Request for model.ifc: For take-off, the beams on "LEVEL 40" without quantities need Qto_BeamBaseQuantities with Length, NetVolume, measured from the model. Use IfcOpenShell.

First a look at what the model holds.

```python
import ifcopenshell
import ifcopenshell.util.element
import ifcopenshell.util.unit

model = ifcopenshell.open("model.ifc")
print(model.schema)
for unit_type in ("LENGTHUNIT", "AREAUNIT", "VOLUMEUNIT"):
    print(unit_type, ifcopenshell.util.unit.calculate_unit_scale(model, unit_type))
storey = next(s for s in model.by_type("IfcBuildingStorey") if s.Name == "LEVEL 40")
beams = [e for e in ifcopenshell.util.element.get_decomposition(storey) if e.is_a("IfcBeam")]
for e in sorted(beams, key=lambda e: e.id()):
    print(e.id(), e.is_a(), e.Name, list(ifcopenshell.util.element.get_psets(e, qtos_only=True)), sep=" | ")
```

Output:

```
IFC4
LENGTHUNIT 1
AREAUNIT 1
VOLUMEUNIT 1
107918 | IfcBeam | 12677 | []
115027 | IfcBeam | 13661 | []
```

```python
import ifcopenshell
import ifcopenshell.api.pset
import ifcopenshell.geom
import ifcopenshell.util.element
import ifcopenshell.util.shape
import ifcopenshell.util.unit

model = ifcopenshell.open("model.ifc")
unit_scale = ifcopenshell.util.unit.calculate_unit_scale(model)
volume_scale = ifcopenshell.util.unit.calculate_unit_scale(model, "VOLUMEUNIT")
settings = ifcopenshell.geom.settings()

storey = next(s for s in model.by_type("IfcBuildingStorey") if s.Name == "LEVEL 40")
beams = [e for e in ifcopenshell.util.element.get_decomposition(storey) if e.is_a("IfcBeam")]

for e in sorted(beams, key=lambda e: e.id()):
    if ifcopenshell.util.element.get_psets(e, qtos_only=True, should_inherit=False):
        continue
    # Geometry comes back in metres, in the element's own axes.
    shape = ifcopenshell.geom.create_shape(settings, e)
    values = {
        "Length": ifcopenshell.util.shape.get_max_xyz(shape.geometry) / unit_scale,
        "NetVolume": ifcopenshell.util.shape.get_volume(shape.geometry) / volume_scale,
    }
    qto = ifcopenshell.api.pset.add_qto(model, product=e, name="Qto_BeamBaseQuantities")
    ifcopenshell.api.pset.edit_qto(model, qto=qto, properties=values)
    print(e.id(), {k: round(v, 3) for k, v in values.items()})

model.write("model_v2.ifc")
```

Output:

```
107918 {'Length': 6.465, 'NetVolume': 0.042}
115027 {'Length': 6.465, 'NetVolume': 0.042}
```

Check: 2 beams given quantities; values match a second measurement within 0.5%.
